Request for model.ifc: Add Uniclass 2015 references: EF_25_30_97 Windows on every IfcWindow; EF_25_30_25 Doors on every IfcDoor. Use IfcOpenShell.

First a look at what the model holds.

```python
import ifcopenshell

model = ifcopenshell.open("model.ifc")
print(model.schema)
print("classifications:", [c.Name for c in model.by_type("IfcClassification")])
for ifc_class in ("IfcDoor", "IfcRoof", "IfcStair", "IfcWall", "IfcWindow"):
    print(ifc_class, len(model.by_type(ifc_class)))
```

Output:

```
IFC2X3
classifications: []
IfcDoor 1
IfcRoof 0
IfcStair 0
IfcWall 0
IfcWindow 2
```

```python
import ifcopenshell
import ifcopenshell.api.classification

model = ifcopenshell.open("model.ifc")

# IFC2X3 requires Source and Edition and has no link from the project to the system.
system = model.create_entity("IfcClassification", Source="NBS", Edition="2015", Name="Uniclass 2015")

codes = {
    "IfcWindow": ("EF_25_30_97", "Windows"),
    "IfcDoor": ("EF_25_30_25", "Doors"),
}
for ifc_class, (code, name) in codes.items():
    products = model.by_type(ifc_class)
    ifcopenshell.api.classification.add_reference(
        model, products=products, classification=system, identification=code, name=name
    )
    print(code, len(products))

model.write("model_rev.ifc")
```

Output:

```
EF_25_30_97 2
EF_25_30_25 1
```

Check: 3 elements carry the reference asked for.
